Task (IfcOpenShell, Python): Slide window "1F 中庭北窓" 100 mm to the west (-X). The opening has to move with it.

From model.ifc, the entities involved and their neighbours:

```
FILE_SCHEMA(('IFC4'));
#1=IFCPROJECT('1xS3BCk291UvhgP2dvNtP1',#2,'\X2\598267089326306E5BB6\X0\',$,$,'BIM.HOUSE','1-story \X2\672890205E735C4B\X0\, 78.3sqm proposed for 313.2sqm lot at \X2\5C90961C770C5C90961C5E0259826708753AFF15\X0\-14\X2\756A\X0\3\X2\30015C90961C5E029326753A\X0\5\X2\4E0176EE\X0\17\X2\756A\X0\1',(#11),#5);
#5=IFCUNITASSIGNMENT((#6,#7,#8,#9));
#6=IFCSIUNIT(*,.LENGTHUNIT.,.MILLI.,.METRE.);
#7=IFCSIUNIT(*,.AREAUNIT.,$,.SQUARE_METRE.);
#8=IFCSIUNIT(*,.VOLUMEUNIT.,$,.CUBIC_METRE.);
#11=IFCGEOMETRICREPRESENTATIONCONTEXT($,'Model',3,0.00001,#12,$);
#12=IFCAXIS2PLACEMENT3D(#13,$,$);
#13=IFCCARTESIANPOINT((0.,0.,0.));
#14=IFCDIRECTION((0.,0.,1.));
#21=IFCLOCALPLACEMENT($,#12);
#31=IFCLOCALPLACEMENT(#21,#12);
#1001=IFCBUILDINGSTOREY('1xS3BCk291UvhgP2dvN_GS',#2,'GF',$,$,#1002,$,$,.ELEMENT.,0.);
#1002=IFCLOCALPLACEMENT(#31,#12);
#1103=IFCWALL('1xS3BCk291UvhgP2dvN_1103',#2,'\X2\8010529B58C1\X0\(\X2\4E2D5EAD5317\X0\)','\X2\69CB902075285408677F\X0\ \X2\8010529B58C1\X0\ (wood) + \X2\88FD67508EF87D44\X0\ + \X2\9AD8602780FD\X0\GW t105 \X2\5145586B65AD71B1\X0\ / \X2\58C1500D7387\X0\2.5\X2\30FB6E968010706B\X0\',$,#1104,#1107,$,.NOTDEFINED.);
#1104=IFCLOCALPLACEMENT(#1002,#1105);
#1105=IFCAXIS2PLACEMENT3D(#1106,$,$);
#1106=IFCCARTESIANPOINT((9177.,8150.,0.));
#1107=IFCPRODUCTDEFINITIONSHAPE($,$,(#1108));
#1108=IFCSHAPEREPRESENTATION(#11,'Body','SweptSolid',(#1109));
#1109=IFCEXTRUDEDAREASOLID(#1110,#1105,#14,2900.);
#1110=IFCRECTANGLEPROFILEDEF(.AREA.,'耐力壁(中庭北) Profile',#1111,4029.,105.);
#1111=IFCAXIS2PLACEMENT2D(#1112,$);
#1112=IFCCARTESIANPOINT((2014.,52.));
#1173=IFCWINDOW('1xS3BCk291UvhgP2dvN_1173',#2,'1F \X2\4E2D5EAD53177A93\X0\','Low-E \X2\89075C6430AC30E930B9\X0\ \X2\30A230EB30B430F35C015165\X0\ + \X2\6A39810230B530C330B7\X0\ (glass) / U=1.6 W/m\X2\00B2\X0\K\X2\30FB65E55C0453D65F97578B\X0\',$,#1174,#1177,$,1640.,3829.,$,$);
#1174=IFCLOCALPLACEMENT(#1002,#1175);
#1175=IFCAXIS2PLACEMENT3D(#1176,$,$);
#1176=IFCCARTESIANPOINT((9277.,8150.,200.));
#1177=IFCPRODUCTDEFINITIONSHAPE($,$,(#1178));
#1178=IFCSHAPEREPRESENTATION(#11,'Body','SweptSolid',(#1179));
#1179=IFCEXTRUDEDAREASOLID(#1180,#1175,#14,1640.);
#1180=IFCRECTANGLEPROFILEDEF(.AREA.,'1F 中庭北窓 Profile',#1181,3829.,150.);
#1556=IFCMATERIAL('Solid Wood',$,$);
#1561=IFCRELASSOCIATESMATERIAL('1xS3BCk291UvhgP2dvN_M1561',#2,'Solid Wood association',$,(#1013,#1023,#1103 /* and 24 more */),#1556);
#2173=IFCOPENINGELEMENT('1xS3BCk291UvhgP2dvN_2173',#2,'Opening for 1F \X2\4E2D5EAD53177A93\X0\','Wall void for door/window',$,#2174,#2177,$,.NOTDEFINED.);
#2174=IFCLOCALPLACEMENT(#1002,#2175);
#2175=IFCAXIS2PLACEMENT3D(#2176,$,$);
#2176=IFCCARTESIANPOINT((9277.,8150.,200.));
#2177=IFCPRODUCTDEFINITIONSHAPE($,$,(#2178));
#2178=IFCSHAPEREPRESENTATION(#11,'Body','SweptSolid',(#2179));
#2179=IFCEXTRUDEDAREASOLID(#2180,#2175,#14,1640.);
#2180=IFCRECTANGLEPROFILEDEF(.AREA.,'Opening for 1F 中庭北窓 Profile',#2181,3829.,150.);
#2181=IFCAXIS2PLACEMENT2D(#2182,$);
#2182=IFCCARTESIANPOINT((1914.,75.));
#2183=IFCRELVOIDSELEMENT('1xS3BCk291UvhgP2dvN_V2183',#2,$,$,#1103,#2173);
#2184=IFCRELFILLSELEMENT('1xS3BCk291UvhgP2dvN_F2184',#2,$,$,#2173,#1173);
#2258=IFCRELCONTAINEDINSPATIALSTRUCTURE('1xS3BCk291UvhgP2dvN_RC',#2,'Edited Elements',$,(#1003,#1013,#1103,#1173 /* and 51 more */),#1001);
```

```python
import ifcopenshell
import ifcopenshell.api.geometry
import ifcopenshell.util.placement

model = ifcopenshell.open("model.ifc")

window = model.by_guid("1xS3BCk291UvhgP2dvN_1173")
opening = window.FillsVoids[0].RelatingOpeningElement
wall = opening.VoidsElements[0].RelatingBuildingElement

wall_matrix = ifcopenshell.util.placement.get_local_placement(wall.ObjectPlacement)
shift = wall_matrix[:3, 0] * -100.0
before = ifcopenshell.util.placement.get_local_placement(window.ObjectPlacement)[:3, 3].copy()

# The window is not placed relative to its opening, so move both.
for product in (opening, window):
    matrix = ifcopenshell.util.placement.get_local_placement(product.ObjectPlacement)
    matrix[:3, 3] += shift
    ifcopenshell.api.geometry.edit_object_placement(model, product=product, matrix=matrix, is_si=False)

after = ifcopenshell.util.placement.get_local_placement(window.ObjectPlacement)[:3, 3]
print("window moved by", (after - before).round(3) + 0.0)

model.write("model_rev.ifc")
```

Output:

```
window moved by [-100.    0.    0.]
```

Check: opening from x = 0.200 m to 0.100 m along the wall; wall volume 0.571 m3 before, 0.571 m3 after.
